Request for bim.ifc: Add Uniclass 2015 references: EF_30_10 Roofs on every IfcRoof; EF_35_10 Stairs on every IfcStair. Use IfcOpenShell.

First a look at what the model holds.

```python
import ifcopenshell

model = ifcopenshell.open("bim.ifc")
print(model.schema)
print("classifications:", [c.Name for c in model.by_type("IfcClassification")])
for ifc_class in ("IfcDoor", "IfcRoof", "IfcStair", "IfcWall", "IfcWindow"):
    print(ifc_class, len(model.by_type(ifc_class)))
```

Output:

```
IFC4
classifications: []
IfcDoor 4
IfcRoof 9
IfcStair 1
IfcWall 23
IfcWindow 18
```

```python
import ifcopenshell
import ifcopenshell.api.classification

model = ifcopenshell.open("bim.ifc")

system = ifcopenshell.api.classification.add_classification(model, classification="Uniclass 2015")

codes = {
    "IfcRoof": ("EF_30_10", "Roofs"),
    "IfcStair": ("EF_35_10", "Stairs"),
}
for ifc_class, (code, name) in codes.items():
    products = model.by_type(ifc_class)
    ifcopenshell.api.classification.add_reference(
        model, products=products, classification=system, identification=code, name=name
    )
    print(code, len(products))

model.write("bim-out.ifc")
```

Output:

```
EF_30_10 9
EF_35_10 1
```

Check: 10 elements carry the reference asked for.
